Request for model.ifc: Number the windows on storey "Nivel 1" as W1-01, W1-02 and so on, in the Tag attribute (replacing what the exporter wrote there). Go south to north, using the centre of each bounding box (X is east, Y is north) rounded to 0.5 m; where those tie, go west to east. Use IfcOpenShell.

First a look at what the model holds.

```python
import ifcopenshell
import ifcopenshell.util.element
import ifcopenshell.util.placement

model = ifcopenshell.open("model.ifc")
print(model.schema)
storey = next(s for s in model.by_type("IfcBuildingStorey") if s.Name == "Nivel 1")
windows = [e for e in ifcopenshell.util.element.get_decomposition(storey) if e.is_a("IfcWindow")]
for e in sorted(windows, key=lambda e: e.id()):
    origin = ifcopenshell.util.placement.get_local_placement(e.ObjectPlacement)[:3, 3]
    print(e.id(), e.Tag, e.Name, origin.round(2) + 0.0, sep=" | ")
```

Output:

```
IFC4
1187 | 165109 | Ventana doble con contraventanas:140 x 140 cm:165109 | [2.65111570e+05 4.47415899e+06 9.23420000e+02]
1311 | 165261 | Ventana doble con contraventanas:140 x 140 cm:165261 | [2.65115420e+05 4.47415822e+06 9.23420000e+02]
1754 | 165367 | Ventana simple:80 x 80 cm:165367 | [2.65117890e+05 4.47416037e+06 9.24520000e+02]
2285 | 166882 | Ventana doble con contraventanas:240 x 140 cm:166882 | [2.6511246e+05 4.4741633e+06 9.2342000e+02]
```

```python
import ifcopenshell
import ifcopenshell.geom
import ifcopenshell.util.element
import ifcopenshell.util.shape

model = ifcopenshell.open("model.ifc")
settings = ifcopenshell.geom.settings()
settings.set("use-world-coords", True)


def centre(element):
    shape = ifcopenshell.geom.create_shape(settings, element)
    return ifcopenshell.util.shape.get_bbox_centroid(shape.geometry)


storey = next(s for s in model.by_type("IfcBuildingStorey") if s.Name == "Nivel 1")
windows = [e for e in ifcopenshell.util.element.get_decomposition(storey) if e.is_a("IfcWindow")]

# Insertion points can sit at a corner or the storey origin, so sort by the geometry (in metres).
centres = {e: centre(e) for e in windows}
windows.sort(key=lambda e: (round(centres[e][1] / 0.5), centres[e][0]))

for i, e in enumerate(windows, start=1):
    number = f"W1-{i:02d}"
    e.Tag = number
    print(e.id(), number)

model.write("model_edited.ifc")
```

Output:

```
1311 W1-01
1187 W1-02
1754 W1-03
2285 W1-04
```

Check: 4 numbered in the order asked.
